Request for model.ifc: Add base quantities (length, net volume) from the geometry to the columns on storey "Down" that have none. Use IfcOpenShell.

First a look at what the model holds.

```python
import ifcopenshell
import ifcopenshell.util.element
import ifcopenshell.util.unit

model = ifcopenshell.open("model.ifc")
print(model.schema)
for unit_type in ("LENGTHUNIT", "AREAUNIT", "VOLUMEUNIT"):
    print(unit_type, ifcopenshell.util.unit.calculate_unit_scale(model, unit_type))
storey = next(s for s in model.by_type("IfcBuildingStorey") if s.Name == "Down")
columns = [e for e in ifcopenshell.util.element.get_decomposition(storey) if e.is_a("IfcColumn")]
for e in sorted(columns, key=lambda e: e.id()):
    print(e.id(), e.is_a(), e.Name, list(ifcopenshell.util.element.get_psets(e, qtos_only=True)), sep=" | ")
```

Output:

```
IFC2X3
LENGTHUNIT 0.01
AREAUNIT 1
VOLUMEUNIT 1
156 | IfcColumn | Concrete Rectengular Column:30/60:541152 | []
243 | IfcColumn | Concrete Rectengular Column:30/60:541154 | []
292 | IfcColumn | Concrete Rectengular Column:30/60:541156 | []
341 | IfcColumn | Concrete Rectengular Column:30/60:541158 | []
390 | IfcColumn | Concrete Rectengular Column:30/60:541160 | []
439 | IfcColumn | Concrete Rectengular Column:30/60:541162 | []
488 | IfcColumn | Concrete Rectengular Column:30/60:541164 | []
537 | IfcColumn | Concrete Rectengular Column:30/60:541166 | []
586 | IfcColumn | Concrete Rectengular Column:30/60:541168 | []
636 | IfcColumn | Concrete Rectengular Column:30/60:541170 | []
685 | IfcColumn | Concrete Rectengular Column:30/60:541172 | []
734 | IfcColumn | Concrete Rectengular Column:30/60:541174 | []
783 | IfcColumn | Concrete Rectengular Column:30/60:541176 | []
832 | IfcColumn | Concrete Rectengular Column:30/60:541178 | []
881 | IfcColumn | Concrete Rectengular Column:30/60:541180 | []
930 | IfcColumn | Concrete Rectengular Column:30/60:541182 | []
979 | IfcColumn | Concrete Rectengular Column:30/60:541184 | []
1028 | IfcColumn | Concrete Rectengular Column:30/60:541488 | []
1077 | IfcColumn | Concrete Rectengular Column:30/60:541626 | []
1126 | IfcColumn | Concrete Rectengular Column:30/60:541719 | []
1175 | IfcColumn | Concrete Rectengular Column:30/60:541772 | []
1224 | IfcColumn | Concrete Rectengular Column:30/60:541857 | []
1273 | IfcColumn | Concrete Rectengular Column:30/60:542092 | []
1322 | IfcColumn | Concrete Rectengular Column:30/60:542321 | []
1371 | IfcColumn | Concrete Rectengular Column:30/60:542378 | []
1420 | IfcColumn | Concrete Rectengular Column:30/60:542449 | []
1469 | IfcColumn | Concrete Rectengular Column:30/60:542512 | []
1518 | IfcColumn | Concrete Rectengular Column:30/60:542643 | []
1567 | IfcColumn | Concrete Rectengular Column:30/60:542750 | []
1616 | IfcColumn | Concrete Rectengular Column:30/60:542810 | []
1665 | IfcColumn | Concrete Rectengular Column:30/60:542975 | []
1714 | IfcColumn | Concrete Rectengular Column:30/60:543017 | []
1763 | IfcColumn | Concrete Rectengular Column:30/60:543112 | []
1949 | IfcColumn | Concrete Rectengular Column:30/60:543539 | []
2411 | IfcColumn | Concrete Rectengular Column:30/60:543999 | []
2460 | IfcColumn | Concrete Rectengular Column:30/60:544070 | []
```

```python
import ifcopenshell
import ifcopenshell.api.pset
import ifcopenshell.geom
import ifcopenshell.util.element
import ifcopenshell.util.shape
import ifcopenshell.util.unit

model = ifcopenshell.open("model.ifc")
unit_scale = ifcopenshell.util.unit.calculate_unit_scale(model)
volume_scale = ifcopenshell.util.unit.calculate_unit_scale(model, "VOLUMEUNIT")
settings = ifcopenshell.geom.settings()

storey = next(s for s in model.by_type("IfcBuildingStorey") if s.Name == "Down")
columns = [e for e in ifcopenshell.util.element.get_decomposition(storey) if e.is_a("IfcColumn")]

for e in sorted(columns, key=lambda e: e.id()):
    if ifcopenshell.util.element.get_psets(e, qtos_only=True, should_inherit=False):
        continue
    # Geometry comes back in metres, in the element's own axes.
    shape = ifcopenshell.geom.create_shape(settings, e)
    values = {
        "Length": ifcopenshell.util.shape.get_z(shape.geometry) / unit_scale,
        "NetVolume": ifcopenshell.util.shape.get_volume(shape.geometry) / volume_scale,
    }
    qto = ifcopenshell.api.pset.add_qto(model, product=e, name="BaseQuantities")
    ifcopenshell.api.pset.edit_qto(model, qto=qto, properties=values)
    print(e.id(), {k: round(v, 3) for k, v in values.items()})

model.write("model_rev.ifc")
```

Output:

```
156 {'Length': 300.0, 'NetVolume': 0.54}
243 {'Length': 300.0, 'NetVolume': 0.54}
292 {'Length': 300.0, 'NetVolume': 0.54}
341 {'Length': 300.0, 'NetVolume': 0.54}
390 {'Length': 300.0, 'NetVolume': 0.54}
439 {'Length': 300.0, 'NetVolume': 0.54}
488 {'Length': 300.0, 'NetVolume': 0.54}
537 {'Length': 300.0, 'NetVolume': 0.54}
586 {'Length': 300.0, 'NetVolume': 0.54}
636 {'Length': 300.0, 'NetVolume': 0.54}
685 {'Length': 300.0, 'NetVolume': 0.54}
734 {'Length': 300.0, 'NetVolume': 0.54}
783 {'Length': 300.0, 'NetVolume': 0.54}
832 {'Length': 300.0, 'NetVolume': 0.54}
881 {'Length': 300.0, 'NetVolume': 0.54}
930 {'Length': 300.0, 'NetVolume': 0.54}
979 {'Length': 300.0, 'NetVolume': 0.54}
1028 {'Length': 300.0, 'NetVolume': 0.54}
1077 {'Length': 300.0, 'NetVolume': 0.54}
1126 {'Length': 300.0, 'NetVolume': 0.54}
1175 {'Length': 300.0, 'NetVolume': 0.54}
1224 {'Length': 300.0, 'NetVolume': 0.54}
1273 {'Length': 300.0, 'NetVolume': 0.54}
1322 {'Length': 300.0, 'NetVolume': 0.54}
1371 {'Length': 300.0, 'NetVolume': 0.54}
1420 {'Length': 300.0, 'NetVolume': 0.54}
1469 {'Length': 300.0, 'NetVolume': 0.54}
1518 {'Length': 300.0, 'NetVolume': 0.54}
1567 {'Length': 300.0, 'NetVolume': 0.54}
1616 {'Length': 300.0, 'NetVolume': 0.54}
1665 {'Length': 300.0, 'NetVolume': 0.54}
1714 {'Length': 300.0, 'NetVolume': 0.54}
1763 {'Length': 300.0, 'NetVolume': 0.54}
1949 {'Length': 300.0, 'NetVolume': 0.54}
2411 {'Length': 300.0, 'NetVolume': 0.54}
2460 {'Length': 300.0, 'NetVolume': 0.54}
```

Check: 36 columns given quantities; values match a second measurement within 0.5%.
